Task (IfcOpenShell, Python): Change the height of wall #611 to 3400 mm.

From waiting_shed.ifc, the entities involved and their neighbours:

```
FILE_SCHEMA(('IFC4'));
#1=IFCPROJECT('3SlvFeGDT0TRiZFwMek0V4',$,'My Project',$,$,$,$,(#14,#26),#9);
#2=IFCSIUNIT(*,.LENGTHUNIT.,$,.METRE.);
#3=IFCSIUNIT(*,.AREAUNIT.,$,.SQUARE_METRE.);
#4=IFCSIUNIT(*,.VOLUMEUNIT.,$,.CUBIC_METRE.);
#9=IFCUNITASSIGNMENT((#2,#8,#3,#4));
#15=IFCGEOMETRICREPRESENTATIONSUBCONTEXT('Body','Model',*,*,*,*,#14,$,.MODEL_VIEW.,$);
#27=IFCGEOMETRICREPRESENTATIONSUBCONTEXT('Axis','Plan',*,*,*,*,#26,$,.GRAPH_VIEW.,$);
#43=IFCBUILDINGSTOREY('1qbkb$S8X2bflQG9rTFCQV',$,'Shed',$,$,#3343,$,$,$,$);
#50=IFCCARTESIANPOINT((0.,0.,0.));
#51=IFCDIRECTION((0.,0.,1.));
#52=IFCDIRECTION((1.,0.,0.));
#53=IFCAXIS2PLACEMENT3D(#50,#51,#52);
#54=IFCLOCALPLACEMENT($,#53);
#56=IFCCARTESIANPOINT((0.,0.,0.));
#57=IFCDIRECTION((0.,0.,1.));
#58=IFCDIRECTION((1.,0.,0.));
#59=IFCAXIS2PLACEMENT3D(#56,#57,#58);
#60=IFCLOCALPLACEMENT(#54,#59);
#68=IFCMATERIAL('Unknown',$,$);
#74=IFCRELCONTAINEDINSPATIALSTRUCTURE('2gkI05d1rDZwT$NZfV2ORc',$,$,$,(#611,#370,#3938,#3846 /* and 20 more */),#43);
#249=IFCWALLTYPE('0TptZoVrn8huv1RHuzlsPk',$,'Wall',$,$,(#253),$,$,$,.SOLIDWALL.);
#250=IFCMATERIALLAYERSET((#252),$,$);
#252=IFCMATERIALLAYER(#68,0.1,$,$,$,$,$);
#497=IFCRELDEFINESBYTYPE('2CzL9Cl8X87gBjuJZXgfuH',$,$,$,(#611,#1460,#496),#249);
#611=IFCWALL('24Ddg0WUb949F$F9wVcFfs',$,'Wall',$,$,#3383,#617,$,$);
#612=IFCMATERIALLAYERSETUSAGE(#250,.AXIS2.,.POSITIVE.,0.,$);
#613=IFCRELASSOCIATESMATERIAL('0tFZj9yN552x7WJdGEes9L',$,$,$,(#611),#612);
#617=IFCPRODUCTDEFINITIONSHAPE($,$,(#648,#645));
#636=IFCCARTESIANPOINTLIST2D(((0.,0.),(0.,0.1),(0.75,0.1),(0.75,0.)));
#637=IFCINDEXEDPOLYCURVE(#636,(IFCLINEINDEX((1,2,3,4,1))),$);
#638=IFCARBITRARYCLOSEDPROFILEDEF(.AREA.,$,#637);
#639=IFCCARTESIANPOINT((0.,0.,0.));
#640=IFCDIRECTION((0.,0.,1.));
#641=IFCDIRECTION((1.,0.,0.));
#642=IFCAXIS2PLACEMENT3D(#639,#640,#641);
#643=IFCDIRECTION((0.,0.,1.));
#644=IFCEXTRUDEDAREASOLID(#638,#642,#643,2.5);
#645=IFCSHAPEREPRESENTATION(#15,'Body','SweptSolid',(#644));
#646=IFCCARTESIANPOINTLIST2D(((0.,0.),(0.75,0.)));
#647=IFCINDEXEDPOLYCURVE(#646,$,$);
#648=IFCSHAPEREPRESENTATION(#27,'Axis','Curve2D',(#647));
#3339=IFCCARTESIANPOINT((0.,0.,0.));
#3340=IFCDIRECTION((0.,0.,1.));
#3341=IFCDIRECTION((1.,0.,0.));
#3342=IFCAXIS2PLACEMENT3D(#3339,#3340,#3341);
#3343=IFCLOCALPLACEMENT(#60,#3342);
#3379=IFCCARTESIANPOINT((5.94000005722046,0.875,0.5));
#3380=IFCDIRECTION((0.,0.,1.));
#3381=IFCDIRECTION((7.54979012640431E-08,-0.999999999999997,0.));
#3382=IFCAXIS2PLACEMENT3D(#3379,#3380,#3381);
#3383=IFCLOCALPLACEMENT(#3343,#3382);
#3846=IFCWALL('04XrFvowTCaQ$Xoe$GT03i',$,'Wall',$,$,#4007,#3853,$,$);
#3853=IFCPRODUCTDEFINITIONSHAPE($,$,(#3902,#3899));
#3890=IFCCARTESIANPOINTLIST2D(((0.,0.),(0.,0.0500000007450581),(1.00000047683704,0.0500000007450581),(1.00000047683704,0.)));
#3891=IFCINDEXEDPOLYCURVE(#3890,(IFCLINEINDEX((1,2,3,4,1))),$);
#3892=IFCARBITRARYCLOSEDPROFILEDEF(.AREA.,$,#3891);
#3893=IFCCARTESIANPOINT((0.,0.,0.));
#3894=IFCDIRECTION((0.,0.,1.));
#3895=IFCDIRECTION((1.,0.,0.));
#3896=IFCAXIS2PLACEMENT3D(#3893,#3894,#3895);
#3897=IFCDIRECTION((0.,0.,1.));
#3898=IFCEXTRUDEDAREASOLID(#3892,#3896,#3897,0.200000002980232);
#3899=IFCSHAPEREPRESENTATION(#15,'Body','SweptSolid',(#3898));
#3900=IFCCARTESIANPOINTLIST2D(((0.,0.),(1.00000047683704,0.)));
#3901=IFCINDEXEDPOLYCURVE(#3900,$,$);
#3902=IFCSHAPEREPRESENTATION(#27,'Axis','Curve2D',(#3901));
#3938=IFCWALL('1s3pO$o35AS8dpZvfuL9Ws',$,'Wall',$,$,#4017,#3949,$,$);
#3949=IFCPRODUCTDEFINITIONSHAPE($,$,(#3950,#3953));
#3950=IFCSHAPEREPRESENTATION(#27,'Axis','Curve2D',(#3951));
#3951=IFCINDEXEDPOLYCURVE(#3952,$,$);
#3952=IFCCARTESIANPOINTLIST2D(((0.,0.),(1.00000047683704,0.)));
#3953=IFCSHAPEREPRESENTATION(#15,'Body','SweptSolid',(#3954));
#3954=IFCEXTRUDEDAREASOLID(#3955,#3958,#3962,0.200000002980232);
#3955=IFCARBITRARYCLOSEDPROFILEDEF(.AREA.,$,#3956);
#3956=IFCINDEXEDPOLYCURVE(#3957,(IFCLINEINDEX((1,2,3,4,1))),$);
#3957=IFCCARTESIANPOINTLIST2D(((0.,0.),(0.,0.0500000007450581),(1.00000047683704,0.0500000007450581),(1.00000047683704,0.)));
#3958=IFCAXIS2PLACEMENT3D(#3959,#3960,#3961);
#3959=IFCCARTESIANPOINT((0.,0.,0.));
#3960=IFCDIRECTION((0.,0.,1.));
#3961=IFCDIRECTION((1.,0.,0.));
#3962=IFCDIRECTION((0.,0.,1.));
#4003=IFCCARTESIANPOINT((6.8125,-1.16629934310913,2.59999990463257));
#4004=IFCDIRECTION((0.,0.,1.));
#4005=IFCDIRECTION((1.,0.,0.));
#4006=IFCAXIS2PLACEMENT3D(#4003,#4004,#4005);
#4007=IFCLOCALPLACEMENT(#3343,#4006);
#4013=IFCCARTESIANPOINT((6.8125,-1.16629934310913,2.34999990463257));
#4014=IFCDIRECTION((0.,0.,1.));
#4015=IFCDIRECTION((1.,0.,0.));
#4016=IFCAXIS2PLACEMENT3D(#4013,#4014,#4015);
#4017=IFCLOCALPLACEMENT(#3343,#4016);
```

```python
import ifcopenshell
import ifcopenshell.geom
import ifcopenshell.util.representation
import ifcopenshell.util.shape
import ifcopenshell.util.unit

model = ifcopenshell.open("waiting_shed.ifc")
unit_scale = ifcopenshell.util.unit.calculate_unit_scale(model)
settings = ifcopenshell.geom.settings()


def volume(element):
    """Net volume in cubic metres, openings subtracted."""
    shape = ifcopenshell.geom.create_shape(settings, element)
    return ifcopenshell.util.shape.get_volume(shape.geometry)


wall = model.by_id(611)
before = volume(wall)

body = ifcopenshell.util.representation.get_representation(wall, "Model", "Body")
solid = body.Items[0]
old_height = solid.Depth
solid.Depth = 3.4 / unit_scale
after = volume(wall)

print(f"height {old_height:g} -> {solid.Depth:g}, volume {before:.3f} -> {after:.3f} m3")

model.write("waiting_shed_rev.ifc")
```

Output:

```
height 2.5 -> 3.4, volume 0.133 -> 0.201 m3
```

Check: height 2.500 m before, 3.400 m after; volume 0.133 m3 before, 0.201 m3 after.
